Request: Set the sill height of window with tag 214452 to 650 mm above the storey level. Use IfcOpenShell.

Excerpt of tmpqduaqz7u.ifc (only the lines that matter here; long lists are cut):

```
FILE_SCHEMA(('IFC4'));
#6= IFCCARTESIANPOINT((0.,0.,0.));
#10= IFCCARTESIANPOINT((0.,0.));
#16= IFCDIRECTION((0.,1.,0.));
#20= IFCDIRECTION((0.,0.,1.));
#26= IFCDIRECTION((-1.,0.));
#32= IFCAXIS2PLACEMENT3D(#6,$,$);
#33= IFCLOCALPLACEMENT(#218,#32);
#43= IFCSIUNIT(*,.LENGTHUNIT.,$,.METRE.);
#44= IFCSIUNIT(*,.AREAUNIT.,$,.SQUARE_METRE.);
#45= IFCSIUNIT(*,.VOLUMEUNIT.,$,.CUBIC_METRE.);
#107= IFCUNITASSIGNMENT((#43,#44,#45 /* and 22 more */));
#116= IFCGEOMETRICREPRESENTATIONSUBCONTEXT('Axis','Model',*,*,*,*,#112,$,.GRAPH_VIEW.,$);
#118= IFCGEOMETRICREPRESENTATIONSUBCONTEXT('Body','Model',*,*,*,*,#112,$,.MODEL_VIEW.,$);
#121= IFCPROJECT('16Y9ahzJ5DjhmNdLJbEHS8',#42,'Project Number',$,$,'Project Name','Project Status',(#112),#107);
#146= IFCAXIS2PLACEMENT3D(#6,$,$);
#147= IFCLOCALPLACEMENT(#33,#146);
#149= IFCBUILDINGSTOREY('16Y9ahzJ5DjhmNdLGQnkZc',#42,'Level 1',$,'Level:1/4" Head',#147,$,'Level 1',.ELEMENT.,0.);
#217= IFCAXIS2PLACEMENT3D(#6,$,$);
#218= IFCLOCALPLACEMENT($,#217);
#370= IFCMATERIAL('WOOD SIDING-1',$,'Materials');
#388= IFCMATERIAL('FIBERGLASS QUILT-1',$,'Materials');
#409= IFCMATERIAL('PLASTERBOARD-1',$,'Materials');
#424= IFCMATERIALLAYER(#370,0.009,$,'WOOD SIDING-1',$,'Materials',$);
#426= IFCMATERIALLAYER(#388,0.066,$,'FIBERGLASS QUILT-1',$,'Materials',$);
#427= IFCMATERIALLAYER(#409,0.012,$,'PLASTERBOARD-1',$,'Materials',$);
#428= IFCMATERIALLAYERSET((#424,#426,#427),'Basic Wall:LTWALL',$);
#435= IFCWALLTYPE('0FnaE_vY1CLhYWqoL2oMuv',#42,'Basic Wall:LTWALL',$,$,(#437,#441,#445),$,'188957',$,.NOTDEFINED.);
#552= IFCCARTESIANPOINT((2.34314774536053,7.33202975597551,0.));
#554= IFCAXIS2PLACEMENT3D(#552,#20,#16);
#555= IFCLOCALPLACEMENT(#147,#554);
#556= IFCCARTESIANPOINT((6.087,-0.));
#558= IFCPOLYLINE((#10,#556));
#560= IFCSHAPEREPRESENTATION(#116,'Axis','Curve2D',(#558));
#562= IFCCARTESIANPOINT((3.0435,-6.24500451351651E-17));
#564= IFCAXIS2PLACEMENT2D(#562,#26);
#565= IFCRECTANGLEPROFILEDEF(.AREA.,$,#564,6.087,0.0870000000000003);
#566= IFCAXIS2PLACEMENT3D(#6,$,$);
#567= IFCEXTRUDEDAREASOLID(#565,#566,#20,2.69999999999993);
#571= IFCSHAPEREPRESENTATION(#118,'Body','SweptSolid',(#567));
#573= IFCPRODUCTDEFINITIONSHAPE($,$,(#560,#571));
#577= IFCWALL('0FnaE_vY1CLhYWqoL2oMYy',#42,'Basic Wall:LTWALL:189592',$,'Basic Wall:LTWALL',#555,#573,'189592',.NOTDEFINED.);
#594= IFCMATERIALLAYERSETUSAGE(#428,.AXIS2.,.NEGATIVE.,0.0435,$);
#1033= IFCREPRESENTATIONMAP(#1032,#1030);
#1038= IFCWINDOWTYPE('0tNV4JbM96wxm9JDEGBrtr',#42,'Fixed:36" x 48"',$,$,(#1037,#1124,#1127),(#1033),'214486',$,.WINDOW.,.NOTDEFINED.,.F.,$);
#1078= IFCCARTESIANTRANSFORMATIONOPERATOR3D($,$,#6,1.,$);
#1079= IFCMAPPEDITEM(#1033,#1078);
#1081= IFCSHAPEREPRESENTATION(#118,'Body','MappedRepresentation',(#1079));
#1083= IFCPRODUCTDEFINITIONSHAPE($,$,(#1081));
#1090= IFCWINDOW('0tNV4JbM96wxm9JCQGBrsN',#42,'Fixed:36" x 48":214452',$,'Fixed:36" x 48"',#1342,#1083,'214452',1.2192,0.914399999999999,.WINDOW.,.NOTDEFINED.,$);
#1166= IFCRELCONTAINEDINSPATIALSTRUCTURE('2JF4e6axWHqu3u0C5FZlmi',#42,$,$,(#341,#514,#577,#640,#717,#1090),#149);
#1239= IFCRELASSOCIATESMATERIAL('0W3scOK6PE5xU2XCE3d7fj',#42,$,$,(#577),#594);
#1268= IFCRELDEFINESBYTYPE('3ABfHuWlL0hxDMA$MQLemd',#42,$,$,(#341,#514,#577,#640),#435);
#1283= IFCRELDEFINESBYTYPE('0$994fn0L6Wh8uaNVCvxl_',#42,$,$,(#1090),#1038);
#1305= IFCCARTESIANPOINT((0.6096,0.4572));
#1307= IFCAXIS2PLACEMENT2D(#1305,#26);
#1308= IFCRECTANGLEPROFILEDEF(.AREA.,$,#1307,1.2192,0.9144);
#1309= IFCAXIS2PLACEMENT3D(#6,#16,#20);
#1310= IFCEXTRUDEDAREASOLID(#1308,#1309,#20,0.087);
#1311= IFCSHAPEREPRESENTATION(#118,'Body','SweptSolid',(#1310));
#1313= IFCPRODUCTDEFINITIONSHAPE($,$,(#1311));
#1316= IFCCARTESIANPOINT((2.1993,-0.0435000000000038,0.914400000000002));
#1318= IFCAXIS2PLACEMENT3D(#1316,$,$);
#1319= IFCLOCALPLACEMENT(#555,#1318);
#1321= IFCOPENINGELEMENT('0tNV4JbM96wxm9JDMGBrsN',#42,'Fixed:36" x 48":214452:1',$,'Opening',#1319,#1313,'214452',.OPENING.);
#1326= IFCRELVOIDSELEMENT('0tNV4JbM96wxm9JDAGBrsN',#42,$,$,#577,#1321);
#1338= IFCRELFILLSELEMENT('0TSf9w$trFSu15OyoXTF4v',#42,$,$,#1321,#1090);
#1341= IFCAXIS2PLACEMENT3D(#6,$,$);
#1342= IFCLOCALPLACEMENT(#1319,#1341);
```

```python
import numpy as np
import ifcopenshell
import ifcopenshell.api.geometry
import ifcopenshell.geom
import ifcopenshell.util.element
import ifcopenshell.util.placement
import ifcopenshell.util.shape
import ifcopenshell.util.unit

model = ifcopenshell.open("tmpqduaqz7u.ifc")
unit_scale = ifcopenshell.util.unit.calculate_unit_scale(model)

window = model.by_guid("0tNV4JbM96wxm9JCQGBrsN")
opening = window.FillsVoids[0].RelatingOpeningElement
storey = ifcopenshell.util.element.get_container(window, ifc_class="IfcBuildingStorey")
level = ifcopenshell.util.placement.get_local_placement(storey.ObjectPlacement)[2, 3]

# The opening's origin need not be at the sill, so measure its lowest point.
shape = ifcopenshell.geom.create_shape(ifcopenshell.geom.settings(), opening)
bottom = ifcopenshell.util.shape.get_shape_bottom_elevation(shape, shape.geometry) / unit_scale
dz = level + 0.65 / unit_scale - bottom

shift = np.array([0.0, 0.0, dz])
# The window is placed relative to its opening, so it follows when the opening moves.
matrix = ifcopenshell.util.placement.get_local_placement(opening.ObjectPlacement)
matrix[:3, 3] += shift
ifcopenshell.api.geometry.edit_object_placement(
    model, product=opening, matrix=matrix, is_si=False, should_transform_children=True
)

print(f"moved by {dz * unit_scale:+.3f} m")

model.write("tmpqduaqz7u_rev.ifc")
```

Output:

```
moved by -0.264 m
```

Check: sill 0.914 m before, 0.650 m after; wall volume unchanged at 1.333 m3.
